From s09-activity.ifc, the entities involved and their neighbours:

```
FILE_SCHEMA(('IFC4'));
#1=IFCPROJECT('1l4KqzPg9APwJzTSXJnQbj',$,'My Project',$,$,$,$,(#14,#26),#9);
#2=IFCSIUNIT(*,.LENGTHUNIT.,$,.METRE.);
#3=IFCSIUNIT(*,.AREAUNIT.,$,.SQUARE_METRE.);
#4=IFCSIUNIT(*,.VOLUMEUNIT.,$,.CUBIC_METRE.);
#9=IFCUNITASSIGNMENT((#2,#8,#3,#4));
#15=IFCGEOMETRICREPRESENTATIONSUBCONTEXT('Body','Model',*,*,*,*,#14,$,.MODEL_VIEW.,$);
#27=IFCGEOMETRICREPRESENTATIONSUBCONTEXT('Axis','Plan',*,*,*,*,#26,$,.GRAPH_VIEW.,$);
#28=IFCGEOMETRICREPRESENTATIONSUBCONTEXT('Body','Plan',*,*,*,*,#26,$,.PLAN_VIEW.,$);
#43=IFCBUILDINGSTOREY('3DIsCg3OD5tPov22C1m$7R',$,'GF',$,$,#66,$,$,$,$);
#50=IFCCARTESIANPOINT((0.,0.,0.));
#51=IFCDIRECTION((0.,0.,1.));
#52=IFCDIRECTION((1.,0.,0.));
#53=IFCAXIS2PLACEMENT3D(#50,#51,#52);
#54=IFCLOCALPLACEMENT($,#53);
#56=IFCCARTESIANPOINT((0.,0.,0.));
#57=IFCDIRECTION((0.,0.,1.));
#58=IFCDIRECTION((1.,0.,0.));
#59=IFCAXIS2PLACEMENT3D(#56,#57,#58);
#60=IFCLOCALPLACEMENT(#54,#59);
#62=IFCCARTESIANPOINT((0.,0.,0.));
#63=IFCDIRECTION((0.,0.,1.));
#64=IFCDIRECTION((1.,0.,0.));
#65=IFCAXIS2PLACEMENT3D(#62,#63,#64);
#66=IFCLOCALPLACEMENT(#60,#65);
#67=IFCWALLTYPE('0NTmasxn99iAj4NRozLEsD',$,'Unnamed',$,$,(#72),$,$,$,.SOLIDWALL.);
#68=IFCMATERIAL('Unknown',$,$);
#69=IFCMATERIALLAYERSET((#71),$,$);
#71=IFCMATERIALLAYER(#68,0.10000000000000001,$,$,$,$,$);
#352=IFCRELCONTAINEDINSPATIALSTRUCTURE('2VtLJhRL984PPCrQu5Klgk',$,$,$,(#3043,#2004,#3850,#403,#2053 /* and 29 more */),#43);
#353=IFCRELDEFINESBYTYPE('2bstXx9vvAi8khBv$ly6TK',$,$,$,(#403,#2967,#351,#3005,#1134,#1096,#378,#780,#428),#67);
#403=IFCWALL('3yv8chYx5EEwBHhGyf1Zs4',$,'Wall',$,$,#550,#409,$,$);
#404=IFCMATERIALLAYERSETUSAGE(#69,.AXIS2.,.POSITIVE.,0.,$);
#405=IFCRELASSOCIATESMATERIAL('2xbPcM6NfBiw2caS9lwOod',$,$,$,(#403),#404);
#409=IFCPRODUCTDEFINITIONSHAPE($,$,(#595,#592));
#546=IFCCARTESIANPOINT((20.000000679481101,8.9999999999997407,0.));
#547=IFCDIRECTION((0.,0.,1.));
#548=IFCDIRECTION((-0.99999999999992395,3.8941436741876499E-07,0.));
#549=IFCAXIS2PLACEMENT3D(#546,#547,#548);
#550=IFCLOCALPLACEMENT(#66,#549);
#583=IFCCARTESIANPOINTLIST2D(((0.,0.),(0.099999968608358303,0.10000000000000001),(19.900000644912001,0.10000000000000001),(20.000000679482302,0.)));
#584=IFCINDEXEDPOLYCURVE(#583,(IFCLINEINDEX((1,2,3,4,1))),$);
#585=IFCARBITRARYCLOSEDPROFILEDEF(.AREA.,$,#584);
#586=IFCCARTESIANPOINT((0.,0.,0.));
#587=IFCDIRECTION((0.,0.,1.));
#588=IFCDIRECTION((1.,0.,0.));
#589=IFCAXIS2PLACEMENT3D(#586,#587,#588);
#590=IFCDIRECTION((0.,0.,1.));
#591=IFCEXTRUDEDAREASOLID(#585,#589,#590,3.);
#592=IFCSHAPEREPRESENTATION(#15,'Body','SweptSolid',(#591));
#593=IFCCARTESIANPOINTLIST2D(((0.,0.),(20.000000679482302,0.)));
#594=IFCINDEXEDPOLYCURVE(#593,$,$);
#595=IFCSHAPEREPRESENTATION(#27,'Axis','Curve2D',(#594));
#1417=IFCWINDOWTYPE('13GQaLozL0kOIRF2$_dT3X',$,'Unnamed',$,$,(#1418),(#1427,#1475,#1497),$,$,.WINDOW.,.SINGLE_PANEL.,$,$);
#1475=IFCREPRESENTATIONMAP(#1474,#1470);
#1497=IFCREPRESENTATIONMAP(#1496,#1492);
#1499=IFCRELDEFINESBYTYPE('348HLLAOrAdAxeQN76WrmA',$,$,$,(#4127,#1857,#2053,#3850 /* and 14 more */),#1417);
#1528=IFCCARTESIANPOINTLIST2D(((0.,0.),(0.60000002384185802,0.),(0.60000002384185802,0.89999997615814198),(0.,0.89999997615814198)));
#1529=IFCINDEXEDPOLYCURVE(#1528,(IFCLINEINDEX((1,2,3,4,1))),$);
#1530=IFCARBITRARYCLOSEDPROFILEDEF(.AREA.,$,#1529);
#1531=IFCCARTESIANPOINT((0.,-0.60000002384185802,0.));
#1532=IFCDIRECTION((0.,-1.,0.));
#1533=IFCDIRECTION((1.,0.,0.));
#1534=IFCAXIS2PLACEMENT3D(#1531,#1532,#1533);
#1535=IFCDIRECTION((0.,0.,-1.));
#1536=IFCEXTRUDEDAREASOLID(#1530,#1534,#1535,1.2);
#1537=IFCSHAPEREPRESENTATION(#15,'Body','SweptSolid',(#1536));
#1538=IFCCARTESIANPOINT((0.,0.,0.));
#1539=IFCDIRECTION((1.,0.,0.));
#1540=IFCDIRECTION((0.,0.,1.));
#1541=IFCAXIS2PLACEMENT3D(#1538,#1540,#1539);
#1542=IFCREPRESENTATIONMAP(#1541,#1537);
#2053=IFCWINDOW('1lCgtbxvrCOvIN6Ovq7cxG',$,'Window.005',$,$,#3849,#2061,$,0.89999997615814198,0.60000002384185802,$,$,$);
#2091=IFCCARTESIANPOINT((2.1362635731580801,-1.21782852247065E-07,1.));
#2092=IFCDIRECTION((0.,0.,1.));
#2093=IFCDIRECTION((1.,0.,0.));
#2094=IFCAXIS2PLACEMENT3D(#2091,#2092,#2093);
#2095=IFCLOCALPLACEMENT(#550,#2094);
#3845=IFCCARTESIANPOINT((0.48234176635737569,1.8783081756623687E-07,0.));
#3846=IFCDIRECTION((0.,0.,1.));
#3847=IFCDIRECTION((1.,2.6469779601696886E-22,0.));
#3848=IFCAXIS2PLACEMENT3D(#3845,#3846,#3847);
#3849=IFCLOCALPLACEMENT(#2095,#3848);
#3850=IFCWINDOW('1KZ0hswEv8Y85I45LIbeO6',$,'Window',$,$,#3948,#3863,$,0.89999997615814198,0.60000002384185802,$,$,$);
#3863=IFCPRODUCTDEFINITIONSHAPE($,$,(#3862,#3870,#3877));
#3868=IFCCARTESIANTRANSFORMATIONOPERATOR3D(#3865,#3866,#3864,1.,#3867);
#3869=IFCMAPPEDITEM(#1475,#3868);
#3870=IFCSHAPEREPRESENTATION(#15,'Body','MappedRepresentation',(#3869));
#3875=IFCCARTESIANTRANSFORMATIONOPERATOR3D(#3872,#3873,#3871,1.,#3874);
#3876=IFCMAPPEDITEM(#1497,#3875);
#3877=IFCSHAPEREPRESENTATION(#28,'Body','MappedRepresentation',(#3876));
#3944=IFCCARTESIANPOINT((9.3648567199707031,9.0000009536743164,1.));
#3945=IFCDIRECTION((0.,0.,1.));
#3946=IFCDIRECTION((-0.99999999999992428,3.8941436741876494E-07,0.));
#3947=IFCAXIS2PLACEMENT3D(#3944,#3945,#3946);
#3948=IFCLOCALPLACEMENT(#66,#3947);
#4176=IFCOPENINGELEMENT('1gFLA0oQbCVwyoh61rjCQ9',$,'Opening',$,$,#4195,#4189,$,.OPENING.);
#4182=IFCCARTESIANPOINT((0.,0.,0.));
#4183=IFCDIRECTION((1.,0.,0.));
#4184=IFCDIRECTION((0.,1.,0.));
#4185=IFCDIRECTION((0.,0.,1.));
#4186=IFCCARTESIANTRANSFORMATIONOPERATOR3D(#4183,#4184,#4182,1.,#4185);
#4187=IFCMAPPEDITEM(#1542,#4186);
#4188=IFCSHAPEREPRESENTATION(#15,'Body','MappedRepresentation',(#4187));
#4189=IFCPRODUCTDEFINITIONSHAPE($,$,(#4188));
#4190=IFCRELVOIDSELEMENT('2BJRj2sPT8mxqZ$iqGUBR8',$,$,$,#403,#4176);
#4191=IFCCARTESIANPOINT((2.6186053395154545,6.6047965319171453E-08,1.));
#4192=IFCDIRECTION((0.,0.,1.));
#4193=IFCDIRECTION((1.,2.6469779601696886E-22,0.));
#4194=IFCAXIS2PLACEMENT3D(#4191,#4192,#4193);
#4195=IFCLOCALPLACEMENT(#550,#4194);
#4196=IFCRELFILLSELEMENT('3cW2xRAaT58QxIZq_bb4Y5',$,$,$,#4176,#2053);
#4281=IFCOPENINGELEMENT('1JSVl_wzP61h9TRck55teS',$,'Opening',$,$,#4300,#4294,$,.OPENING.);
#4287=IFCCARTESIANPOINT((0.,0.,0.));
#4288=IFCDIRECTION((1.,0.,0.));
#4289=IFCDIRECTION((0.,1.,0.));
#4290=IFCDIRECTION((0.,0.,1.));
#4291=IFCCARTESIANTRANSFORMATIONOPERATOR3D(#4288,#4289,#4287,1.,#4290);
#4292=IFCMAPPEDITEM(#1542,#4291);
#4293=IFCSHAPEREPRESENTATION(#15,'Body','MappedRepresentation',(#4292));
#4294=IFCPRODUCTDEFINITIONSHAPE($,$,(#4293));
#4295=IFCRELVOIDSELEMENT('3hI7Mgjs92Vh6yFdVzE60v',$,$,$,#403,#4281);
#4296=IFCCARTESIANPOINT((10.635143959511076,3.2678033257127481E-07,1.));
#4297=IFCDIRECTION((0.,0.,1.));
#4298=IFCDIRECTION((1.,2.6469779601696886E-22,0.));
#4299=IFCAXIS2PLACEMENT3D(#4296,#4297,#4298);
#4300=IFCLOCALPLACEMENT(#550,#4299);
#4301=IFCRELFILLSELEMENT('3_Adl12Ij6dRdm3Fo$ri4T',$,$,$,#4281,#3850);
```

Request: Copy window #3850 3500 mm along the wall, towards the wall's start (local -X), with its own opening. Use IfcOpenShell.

```python
import ifcopenshell
import ifcopenshell.api.feature
import ifcopenshell.api.geometry
import ifcopenshell.api.root
import ifcopenshell.geom
import ifcopenshell.util.element
import ifcopenshell.util.placement
import ifcopenshell.util.shape

model = ifcopenshell.open("s09-activity.ifc")
settings = ifcopenshell.geom.settings()


def volume(element):
    """Net volume in cubic metres, openings subtracted."""
    shape = ifcopenshell.geom.create_shape(settings, element)
    return ifcopenshell.util.shape.get_volume(shape.geometry)


window = model.by_guid("1KZ0hswEv8Y85I45LIbeO6")
opening = window.FillsVoids[0].RelatingOpeningElement
wall = opening.VoidsElements[0].RelatingBuildingElement
before = volume(wall)
shift = ifcopenshell.util.placement.get_local_placement(wall.ObjectPlacement)[:3, 0] * -3.5

# copy_class copies the void relationship, type, container and properties, but no geometry.
new_opening = ifcopenshell.api.root.copy_class(model, product=opening)
new_opening.Representation = ifcopenshell.util.element.copy_deep(
    model, opening.Representation, exclude=["IfcGeometricRepresentationContext", "IfcRepresentationMap"]
)
new_window = ifcopenshell.api.root.copy_class(model, product=window)
new_window.Representation = ifcopenshell.util.element.copy_deep(
    model, window.Representation, exclude=["IfcGeometricRepresentationContext", "IfcRepresentationMap"]
)
ifcopenshell.api.feature.add_filling(model, opening=new_opening, element=new_window)

for old, new in ((opening, new_opening), (window, new_window)):
    matrix = ifcopenshell.util.placement.get_local_placement(old.ObjectPlacement)
    matrix[:3, 3] += shift
    ifcopenshell.api.geometry.edit_object_placement(model, product=new, matrix=matrix, is_si=False)

after = volume(wall)

print(f"wall volume {before:.3f} -> {after:.3f} m3")

model.write("s09-activity_updated.ifc")
```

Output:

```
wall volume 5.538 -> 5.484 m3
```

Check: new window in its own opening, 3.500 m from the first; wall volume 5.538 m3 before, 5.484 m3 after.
